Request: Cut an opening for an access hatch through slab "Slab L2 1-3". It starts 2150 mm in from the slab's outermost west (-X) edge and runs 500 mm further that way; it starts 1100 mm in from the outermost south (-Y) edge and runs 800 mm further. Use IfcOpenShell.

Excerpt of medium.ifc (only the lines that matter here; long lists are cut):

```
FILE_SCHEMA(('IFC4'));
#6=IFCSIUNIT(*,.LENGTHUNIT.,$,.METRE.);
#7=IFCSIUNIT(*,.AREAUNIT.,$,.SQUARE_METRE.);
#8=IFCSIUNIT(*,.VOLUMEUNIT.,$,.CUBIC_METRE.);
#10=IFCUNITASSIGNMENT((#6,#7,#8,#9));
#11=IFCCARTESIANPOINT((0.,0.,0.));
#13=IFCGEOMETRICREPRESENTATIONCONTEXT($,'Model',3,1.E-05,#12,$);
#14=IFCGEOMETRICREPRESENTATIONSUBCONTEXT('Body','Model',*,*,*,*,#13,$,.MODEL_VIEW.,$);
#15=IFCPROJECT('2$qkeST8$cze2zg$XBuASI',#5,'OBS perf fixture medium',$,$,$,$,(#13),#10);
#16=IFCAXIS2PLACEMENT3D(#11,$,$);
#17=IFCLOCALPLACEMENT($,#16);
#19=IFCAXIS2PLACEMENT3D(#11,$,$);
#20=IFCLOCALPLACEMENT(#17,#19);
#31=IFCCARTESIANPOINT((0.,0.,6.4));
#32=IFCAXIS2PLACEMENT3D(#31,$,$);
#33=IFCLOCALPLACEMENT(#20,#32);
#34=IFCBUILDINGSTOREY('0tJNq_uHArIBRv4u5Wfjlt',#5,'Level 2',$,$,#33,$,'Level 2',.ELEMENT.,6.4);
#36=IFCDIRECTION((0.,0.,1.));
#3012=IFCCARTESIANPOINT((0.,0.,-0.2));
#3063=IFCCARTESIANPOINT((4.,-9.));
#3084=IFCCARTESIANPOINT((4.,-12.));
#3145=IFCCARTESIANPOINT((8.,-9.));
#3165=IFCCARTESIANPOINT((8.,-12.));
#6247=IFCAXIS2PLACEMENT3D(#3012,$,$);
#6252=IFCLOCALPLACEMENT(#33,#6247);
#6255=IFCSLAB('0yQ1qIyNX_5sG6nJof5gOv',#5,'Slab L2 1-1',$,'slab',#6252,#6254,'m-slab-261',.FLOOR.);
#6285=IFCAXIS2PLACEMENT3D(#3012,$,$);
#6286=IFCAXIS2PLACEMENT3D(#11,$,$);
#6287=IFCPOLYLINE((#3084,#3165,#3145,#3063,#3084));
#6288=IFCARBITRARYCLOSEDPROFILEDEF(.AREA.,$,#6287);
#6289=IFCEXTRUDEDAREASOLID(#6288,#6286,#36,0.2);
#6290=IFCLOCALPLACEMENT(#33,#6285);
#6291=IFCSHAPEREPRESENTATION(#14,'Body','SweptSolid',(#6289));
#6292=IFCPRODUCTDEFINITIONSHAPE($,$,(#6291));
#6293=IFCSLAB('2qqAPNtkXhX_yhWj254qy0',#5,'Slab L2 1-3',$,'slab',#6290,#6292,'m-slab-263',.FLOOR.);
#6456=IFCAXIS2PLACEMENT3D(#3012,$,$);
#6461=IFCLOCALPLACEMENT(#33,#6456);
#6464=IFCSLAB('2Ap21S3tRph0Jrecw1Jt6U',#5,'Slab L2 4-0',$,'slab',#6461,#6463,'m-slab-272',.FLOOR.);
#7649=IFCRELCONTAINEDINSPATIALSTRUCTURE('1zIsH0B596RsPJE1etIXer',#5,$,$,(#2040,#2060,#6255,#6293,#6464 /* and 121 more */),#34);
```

```python
import numpy as np
import ifcopenshell
import ifcopenshell.api.feature
import ifcopenshell.api.geometry
import ifcopenshell.api.root
import ifcopenshell.geom
import ifcopenshell.util.placement
import ifcopenshell.util.representation
import ifcopenshell.util.shape
import ifcopenshell.util.unit

model = ifcopenshell.open("medium.ifc")
unit_scale = ifcopenshell.util.unit.calculate_unit_scale(model)
settings = ifcopenshell.geom.settings()


def volume(element):
    """Net volume in cubic metres, openings subtracted."""
    shape = ifcopenshell.geom.create_shape(settings, element)
    return ifcopenshell.util.shape.get_volume(shape.geometry)


slab = model.by_guid("2qqAPNtkXhX_yhWj254qy0")
before = volume(slab)

# Extent in the slab's own axes, in metres. The edges named are its -X and -Y sides.
slab_shape = ifcopenshell.geom.create_shape(settings, slab)
vertices = ifcopenshell.util.shape.get_vertices(slab_shape.geometry)
x_min, y_min, bottom = vertices.min(axis=0)
top = vertices[:, 2].max()

opening = ifcopenshell.api.root.create_entity(model, ifc_class="IfcOpeningElement", name="Access hatch opening", predefined_type="OPENING")
context = ifcopenshell.util.representation.get_context(model, "Model", "Body", "MODEL_VIEW")
width, depth = 0.5, 0.8
outline = [(0.0, 0.0), (width, 0.0), (width, depth), (0.0, depth), (0.0, 0.0)]
# Overshoot both faces by 50 mm so the cut is clean.
shape = ifcopenshell.api.geometry.add_slab_representation(
    model, context=context, depth=top - bottom + 0.1, polyline=outline
)
ifcopenshell.api.geometry.assign_representation(model, product=opening, representation=shape)

matrix = ifcopenshell.util.placement.get_local_placement(slab.ObjectPlacement)
matrix[:, 3] = matrix @ np.append(np.array([x_min + 2.15, y_min + 1.1, bottom - 0.05]) / unit_scale, 1.0)
ifcopenshell.api.geometry.edit_object_placement(model, product=opening, matrix=matrix, is_si=False)
ifcopenshell.api.feature.add_feature(model, feature=opening, element=slab)

after = volume(slab)

print(f"slab volume {before:.3f} -> {after:.3f} m3")

model.write("medium_edited.ifc")
```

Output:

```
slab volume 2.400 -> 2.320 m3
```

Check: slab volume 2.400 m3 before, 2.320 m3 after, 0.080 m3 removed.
